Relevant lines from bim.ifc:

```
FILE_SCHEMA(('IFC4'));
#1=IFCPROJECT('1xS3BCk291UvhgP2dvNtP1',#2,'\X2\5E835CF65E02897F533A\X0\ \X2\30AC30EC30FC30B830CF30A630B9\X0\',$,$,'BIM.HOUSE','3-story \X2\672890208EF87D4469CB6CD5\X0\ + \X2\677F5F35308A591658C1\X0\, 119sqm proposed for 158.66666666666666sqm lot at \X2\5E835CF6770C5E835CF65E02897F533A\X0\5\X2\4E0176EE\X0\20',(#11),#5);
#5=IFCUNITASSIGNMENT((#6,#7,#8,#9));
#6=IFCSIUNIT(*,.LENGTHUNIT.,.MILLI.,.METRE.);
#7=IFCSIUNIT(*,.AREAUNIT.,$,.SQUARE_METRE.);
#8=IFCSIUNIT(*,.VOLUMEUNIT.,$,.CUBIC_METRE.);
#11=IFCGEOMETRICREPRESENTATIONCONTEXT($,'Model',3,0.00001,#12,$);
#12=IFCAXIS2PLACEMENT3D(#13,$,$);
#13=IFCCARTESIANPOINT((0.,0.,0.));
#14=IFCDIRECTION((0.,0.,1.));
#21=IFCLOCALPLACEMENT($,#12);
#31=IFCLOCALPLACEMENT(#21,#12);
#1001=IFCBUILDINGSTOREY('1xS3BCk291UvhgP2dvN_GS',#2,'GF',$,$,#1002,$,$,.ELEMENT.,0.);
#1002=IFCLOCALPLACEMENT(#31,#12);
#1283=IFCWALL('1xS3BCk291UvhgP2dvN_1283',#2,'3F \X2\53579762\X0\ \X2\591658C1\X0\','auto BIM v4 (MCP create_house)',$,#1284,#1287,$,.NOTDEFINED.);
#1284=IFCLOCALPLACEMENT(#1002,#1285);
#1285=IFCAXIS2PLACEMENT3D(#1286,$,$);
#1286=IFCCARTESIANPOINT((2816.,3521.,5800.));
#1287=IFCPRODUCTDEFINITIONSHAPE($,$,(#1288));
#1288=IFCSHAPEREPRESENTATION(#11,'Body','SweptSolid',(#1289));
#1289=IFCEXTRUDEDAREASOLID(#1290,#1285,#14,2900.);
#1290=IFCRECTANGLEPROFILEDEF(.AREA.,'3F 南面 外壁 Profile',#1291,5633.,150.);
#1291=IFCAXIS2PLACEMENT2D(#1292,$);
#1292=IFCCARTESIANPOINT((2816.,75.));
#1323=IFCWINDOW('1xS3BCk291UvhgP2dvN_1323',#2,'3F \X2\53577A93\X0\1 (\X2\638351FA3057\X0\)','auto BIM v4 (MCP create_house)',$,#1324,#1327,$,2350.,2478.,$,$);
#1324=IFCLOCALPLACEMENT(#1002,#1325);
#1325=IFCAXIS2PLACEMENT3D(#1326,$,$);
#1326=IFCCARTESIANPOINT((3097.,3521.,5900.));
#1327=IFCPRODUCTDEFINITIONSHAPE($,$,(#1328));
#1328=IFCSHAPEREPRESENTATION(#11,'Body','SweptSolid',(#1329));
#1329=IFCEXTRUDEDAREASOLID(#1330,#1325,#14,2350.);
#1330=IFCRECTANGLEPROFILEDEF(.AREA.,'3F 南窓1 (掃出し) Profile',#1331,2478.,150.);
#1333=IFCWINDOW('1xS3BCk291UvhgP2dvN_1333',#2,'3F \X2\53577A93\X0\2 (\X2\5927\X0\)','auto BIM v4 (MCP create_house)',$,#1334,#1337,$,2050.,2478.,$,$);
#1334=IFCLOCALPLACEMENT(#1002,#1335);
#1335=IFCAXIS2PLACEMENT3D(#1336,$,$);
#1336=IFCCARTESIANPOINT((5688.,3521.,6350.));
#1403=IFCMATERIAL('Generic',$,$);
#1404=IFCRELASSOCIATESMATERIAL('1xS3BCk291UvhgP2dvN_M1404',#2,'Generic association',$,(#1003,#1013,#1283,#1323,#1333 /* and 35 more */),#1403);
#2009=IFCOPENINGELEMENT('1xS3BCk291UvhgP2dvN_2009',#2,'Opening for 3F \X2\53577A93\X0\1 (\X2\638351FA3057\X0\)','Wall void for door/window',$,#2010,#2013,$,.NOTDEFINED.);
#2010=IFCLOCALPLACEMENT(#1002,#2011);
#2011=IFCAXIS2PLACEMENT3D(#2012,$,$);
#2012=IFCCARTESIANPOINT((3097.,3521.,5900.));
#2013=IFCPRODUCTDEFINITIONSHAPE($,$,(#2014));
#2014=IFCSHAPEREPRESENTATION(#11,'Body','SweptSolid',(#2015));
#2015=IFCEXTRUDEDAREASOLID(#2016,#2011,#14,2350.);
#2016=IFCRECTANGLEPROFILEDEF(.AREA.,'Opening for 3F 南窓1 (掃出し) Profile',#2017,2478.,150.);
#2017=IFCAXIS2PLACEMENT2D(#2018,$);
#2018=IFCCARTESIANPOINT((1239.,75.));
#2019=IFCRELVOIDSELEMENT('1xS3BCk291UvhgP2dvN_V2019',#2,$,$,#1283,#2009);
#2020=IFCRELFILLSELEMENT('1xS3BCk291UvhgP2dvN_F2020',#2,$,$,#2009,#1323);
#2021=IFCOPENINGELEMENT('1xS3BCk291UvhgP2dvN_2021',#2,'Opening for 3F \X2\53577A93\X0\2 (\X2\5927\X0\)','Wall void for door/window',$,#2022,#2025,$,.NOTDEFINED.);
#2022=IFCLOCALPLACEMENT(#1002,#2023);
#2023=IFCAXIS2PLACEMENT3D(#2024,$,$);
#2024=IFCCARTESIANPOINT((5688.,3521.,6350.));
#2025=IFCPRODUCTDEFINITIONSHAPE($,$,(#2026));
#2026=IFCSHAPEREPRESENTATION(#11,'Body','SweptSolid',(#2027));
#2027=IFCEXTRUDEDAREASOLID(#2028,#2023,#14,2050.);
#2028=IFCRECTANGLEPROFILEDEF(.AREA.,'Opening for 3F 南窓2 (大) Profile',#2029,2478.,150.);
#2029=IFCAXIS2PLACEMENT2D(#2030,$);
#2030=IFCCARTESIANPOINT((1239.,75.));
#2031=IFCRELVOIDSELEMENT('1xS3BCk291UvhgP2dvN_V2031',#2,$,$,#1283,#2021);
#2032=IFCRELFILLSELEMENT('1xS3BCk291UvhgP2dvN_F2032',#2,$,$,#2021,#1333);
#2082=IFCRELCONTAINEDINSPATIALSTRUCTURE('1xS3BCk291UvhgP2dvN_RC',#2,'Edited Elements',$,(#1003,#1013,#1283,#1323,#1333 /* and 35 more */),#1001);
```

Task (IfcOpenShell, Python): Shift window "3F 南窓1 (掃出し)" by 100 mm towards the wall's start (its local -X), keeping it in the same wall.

```python
import ifcopenshell
import ifcopenshell.api.geometry
import ifcopenshell.util.placement
import ifcopenshell.util.unit

model = ifcopenshell.open("bim.ifc")
unit_scale = ifcopenshell.util.unit.calculate_unit_scale(model)

window = model.by_guid("1xS3BCk291UvhgP2dvN_1323")
opening = window.FillsVoids[0].RelatingOpeningElement
wall = opening.VoidsElements[0].RelatingBuildingElement

wall_matrix = ifcopenshell.util.placement.get_local_placement(wall.ObjectPlacement)
shift = wall_matrix[:3, 0] * -0.1 / unit_scale
before = ifcopenshell.util.placement.get_local_placement(window.ObjectPlacement)[:3, 3].copy()

# The window is not placed relative to its opening, so move both.
for product in (opening, window):
    matrix = ifcopenshell.util.placement.get_local_placement(product.ObjectPlacement)
    matrix[:3, 3] += shift
    ifcopenshell.api.geometry.edit_object_placement(model, product=product, matrix=matrix, is_si=False)

after = ifcopenshell.util.placement.get_local_placement(window.ObjectPlacement)[:3, 3]
print("window moved by", (after - before).round(3) + 0.0)

model.write("bim_v2.ifc")
```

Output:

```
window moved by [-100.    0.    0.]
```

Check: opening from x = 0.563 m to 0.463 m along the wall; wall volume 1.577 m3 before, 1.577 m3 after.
